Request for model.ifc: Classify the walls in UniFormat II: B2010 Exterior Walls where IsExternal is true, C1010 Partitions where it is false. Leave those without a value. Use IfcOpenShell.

First a look at what the model holds.

```python
import ifcopenshell
import ifcopenshell.util.element

model = ifcopenshell.open("model.ifc")
print(model.schema)
print("classifications:", [c.Name for c in model.by_type("IfcClassification")])
values = [ifcopenshell.util.element.get_pset(e, "Pset_WallCommon", "IsExternal") for e in model.by_type("IfcWall")]
for value in (True, False, None):
    print("IsExternal", value, values.count(value))
```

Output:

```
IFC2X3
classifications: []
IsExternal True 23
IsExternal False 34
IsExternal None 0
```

```python
import ifcopenshell
import ifcopenshell.api.classification
import ifcopenshell.util.element

model = ifcopenshell.open("model.ifc")

# IFC2X3 requires Source and Edition and has no link from the project to the system.
system = model.create_entity("IfcClassification", Source="ASTM", Edition="E1557", Name="UniFormat II")

walls = model.by_type("IfcWall")
external = {e: ifcopenshell.util.element.get_pset(e, "Pset_WallCommon", "IsExternal") for e in walls}
for flag, code, name in ((True, "B2010", "Exterior Walls"), (False, "C1010", "Partitions")):
    products = [e for e in walls if external[e] is flag]
    ifcopenshell.api.classification.add_reference(
        model, products=products, classification=system, identification=code, name=name
    )
    print(code, len(products))

model.write("model_v2.ifc")
```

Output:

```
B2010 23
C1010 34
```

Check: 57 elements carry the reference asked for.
